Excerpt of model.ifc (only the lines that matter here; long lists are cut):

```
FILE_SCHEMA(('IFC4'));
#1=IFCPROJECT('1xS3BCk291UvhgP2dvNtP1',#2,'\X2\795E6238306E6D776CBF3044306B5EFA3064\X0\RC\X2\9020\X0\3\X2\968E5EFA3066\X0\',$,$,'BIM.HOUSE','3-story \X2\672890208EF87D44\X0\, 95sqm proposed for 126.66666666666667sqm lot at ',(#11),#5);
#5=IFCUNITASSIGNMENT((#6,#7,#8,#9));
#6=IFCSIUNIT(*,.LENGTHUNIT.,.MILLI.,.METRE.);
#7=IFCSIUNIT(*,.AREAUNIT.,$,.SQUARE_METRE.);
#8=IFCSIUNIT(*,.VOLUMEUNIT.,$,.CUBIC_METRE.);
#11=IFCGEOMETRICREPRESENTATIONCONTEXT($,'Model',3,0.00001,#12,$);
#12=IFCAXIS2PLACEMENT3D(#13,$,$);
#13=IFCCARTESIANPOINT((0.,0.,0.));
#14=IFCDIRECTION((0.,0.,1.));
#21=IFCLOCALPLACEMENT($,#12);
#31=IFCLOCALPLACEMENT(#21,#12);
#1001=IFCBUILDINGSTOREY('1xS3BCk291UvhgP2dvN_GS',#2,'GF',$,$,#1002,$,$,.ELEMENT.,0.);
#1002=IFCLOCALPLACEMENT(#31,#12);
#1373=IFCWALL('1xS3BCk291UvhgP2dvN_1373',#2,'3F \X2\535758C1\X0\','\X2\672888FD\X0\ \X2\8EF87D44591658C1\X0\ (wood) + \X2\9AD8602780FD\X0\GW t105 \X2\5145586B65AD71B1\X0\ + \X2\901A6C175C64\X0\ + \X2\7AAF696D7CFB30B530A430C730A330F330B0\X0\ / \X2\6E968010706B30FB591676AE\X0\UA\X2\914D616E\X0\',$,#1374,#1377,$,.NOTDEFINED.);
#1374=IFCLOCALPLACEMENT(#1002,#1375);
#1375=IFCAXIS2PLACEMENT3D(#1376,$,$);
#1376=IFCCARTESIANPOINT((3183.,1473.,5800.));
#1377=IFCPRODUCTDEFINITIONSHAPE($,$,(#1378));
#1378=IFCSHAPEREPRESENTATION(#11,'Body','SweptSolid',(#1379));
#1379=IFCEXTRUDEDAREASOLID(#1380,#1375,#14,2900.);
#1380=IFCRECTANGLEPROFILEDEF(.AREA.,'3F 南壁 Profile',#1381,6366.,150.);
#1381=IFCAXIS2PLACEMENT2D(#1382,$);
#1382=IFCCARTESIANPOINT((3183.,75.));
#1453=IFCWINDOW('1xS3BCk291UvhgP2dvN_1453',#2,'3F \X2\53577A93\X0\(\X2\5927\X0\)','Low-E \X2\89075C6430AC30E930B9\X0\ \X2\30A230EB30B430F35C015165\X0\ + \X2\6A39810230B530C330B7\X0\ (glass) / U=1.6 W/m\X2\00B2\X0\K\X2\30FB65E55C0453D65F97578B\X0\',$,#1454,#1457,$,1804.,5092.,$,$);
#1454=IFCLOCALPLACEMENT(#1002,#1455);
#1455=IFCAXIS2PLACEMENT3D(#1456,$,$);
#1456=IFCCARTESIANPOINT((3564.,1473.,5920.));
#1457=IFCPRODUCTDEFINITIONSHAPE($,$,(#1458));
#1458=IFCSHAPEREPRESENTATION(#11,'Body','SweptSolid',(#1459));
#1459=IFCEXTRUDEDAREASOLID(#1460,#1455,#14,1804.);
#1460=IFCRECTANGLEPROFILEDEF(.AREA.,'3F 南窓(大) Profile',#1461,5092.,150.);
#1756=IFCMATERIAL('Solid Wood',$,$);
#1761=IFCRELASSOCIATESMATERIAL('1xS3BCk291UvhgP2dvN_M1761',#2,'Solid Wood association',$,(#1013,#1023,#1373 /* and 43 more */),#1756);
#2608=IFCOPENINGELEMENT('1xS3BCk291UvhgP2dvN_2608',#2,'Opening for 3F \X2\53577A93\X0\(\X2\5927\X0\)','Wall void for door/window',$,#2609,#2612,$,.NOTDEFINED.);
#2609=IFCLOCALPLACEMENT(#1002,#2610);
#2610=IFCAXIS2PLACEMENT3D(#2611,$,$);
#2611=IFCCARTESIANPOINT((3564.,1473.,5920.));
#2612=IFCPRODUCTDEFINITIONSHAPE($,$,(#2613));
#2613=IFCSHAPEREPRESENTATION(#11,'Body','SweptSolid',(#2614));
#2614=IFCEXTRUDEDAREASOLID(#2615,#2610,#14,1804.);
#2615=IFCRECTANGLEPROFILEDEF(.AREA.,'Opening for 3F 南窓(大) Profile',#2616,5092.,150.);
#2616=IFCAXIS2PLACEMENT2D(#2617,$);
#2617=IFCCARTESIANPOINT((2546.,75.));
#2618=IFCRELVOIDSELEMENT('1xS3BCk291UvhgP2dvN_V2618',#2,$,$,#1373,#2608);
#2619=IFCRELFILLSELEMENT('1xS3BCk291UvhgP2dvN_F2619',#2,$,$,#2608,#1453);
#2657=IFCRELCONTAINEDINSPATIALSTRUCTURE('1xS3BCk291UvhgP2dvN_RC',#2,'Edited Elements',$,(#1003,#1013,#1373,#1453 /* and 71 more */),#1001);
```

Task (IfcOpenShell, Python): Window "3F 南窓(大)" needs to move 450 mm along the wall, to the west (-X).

```python
import ifcopenshell
import ifcopenshell.api.geometry
import ifcopenshell.util.placement
import ifcopenshell.util.unit

model = ifcopenshell.open("model.ifc")
unit_scale = ifcopenshell.util.unit.calculate_unit_scale(model)

window = model.by_id(1453)
opening = window.FillsVoids[0].RelatingOpeningElement
wall = opening.VoidsElements[0].RelatingBuildingElement

wall_matrix = ifcopenshell.util.placement.get_local_placement(wall.ObjectPlacement)
shift = wall_matrix[:3, 0] * -0.45 / unit_scale
before = ifcopenshell.util.placement.get_local_placement(window.ObjectPlacement)[:3, 3].copy()

# The window is not placed relative to its opening, so move both.
for product in (opening, window):
    matrix = ifcopenshell.util.placement.get_local_placement(product.ObjectPlacement)
    matrix[:3, 3] += shift
    ifcopenshell.api.geometry.edit_object_placement(model, product=product, matrix=matrix, is_si=False)

after = ifcopenshell.util.placement.get_local_placement(window.ObjectPlacement)[:3, 3]
print("window moved by", (after - before).round(3) + 0.0)

model.write("model_rev.ifc")
```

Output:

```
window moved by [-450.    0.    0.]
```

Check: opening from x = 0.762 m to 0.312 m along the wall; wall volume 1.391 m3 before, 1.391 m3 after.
